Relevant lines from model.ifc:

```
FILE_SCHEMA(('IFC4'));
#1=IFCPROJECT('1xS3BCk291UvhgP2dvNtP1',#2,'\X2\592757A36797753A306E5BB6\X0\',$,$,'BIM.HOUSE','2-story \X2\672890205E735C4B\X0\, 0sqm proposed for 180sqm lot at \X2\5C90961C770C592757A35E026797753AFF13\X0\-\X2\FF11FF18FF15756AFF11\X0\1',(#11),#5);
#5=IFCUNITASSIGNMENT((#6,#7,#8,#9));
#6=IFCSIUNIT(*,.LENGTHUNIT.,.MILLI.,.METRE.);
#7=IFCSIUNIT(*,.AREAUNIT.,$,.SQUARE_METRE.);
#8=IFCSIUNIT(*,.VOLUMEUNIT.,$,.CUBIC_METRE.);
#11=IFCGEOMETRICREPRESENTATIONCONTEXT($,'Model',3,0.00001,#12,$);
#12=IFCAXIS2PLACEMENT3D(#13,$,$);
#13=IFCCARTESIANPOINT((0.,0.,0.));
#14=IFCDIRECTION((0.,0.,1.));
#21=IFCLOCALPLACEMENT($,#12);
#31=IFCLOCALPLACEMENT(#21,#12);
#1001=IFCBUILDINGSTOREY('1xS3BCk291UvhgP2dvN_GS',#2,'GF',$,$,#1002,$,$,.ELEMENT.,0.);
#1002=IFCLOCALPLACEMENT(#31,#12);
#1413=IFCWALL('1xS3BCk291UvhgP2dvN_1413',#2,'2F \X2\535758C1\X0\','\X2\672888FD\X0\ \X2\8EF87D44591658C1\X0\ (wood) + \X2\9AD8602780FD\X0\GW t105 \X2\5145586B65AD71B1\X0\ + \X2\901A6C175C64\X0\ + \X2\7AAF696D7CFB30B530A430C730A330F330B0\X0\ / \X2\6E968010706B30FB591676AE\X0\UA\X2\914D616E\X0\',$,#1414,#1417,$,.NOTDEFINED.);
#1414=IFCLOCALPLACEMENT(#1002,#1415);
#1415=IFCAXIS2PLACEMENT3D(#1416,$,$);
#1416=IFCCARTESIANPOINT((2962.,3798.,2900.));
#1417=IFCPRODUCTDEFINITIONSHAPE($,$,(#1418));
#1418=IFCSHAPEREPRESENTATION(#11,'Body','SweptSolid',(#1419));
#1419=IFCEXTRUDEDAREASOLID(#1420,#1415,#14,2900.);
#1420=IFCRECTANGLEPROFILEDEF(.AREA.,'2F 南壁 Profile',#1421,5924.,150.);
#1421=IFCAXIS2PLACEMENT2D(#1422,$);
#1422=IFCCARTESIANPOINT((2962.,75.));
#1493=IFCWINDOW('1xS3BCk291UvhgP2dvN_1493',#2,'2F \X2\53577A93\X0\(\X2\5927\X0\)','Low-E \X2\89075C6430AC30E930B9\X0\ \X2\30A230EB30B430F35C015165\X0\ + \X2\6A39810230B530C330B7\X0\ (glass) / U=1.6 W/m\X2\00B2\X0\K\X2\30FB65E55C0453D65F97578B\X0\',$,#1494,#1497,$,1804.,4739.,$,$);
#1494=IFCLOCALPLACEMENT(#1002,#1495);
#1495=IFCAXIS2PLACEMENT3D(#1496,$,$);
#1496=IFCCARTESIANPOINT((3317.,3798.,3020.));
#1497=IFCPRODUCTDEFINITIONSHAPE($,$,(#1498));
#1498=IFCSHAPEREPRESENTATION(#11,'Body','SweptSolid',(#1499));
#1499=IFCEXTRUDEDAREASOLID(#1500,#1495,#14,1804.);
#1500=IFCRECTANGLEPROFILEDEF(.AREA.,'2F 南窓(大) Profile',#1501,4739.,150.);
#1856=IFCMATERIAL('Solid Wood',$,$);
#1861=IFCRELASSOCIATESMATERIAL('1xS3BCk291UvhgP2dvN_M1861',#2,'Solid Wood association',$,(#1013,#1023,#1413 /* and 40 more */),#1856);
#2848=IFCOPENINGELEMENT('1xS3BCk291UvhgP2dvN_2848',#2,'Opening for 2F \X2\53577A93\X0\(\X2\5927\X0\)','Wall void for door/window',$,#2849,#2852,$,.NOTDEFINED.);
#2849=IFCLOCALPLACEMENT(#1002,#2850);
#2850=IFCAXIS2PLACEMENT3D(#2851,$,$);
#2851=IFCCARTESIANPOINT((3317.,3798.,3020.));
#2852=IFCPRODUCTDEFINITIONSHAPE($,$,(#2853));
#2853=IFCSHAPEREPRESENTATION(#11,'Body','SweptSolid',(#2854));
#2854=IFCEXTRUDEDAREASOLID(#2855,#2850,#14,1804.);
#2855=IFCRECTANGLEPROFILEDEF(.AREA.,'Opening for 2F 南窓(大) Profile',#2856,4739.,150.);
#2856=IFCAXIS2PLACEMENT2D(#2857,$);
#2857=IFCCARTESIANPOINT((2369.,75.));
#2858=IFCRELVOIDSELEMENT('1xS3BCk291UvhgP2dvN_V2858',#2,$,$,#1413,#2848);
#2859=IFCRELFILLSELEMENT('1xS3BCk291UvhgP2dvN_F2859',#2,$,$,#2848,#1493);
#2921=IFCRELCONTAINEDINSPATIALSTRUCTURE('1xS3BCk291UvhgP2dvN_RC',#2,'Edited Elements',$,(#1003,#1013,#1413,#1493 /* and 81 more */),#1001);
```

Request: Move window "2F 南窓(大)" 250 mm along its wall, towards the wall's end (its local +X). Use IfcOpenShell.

```python
import ifcopenshell
import ifcopenshell.api.geometry
import ifcopenshell.util.placement

model = ifcopenshell.open("model.ifc")

window = model.by_id(1493)
opening = window.FillsVoids[0].RelatingOpeningElement
wall = opening.VoidsElements[0].RelatingBuildingElement

wall_matrix = ifcopenshell.util.placement.get_local_placement(wall.ObjectPlacement)
shift = wall_matrix[:3, 0] * 250.0
before = ifcopenshell.util.placement.get_local_placement(window.ObjectPlacement)[:3, 3].copy()

# The window is not placed relative to its opening, so move both.
for product in (opening, window):
    matrix = ifcopenshell.util.placement.get_local_placement(product.ObjectPlacement)
    matrix[:3, 3] += shift
    ifcopenshell.api.geometry.edit_object_placement(model, product=product, matrix=matrix, is_si=False)

after = ifcopenshell.util.placement.get_local_placement(window.ObjectPlacement)[:3, 3]
print("window moved by", (after - before).round(3) + 0.0)

model.write("model_updated.ifc")
```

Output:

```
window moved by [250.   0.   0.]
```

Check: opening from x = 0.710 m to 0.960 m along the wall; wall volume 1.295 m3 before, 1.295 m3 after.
